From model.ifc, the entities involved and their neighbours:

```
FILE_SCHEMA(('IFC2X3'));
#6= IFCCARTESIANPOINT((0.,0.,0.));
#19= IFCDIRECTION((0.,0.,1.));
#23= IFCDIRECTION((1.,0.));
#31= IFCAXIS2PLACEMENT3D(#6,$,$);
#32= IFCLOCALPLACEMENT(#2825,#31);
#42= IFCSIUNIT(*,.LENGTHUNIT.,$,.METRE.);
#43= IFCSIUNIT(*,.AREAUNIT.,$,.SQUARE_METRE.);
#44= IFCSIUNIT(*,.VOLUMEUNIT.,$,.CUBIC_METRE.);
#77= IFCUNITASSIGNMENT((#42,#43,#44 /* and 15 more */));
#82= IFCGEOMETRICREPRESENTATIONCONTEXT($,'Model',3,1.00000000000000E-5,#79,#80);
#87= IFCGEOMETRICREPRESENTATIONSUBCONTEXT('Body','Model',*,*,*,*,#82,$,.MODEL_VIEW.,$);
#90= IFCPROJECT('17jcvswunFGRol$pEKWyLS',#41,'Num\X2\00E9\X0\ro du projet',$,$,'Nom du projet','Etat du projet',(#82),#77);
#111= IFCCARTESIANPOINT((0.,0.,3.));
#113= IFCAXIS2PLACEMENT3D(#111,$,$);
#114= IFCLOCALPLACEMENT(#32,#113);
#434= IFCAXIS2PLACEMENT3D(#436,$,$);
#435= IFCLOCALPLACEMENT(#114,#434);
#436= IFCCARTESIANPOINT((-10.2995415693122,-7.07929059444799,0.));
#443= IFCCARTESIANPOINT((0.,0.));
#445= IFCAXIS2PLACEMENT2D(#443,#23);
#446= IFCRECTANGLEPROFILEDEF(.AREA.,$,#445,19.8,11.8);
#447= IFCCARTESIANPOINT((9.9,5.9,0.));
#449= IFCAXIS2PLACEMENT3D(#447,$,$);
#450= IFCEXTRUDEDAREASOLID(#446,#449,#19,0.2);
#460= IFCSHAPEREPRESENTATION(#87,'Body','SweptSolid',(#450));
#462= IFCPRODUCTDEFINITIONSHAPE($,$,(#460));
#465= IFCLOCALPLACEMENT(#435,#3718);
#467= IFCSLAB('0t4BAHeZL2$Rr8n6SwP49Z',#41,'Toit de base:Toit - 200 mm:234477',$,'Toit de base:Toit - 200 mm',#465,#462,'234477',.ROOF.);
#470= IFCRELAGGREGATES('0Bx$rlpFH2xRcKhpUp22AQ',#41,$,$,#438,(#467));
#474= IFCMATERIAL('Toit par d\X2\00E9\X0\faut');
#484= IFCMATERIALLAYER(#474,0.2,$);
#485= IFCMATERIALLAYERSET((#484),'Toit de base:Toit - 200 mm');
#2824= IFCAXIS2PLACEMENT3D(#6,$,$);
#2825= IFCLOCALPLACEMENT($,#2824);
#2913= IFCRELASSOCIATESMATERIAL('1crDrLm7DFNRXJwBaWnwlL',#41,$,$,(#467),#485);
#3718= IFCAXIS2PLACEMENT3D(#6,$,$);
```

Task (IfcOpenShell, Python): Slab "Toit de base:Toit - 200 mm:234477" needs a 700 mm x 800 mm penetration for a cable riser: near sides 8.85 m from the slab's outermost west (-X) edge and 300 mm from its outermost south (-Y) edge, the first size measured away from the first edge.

```python
import numpy as np
import ifcopenshell
import ifcopenshell.api.feature
import ifcopenshell.api.geometry
import ifcopenshell.api.root
import ifcopenshell.geom
import ifcopenshell.util.placement
import ifcopenshell.util.representation
import ifcopenshell.util.shape
import ifcopenshell.util.unit

model = ifcopenshell.open("model.ifc")
unit_scale = ifcopenshell.util.unit.calculate_unit_scale(model)
settings = ifcopenshell.geom.settings()


def volume(element):
    """Net volume in cubic metres, openings subtracted."""
    shape = ifcopenshell.geom.create_shape(settings, element)
    return ifcopenshell.util.shape.get_volume(shape.geometry)


slab = model.by_id(467)
before = volume(slab)

# Extent in the slab's own axes, in metres. The edges named are its -X and -Y sides.
slab_shape = ifcopenshell.geom.create_shape(settings, slab)
vertices = ifcopenshell.util.shape.get_vertices(slab_shape.geometry)
x_min, y_min, bottom = vertices.min(axis=0)
top = vertices[:, 2].max()

opening = ifcopenshell.api.root.create_entity(model, ifc_class="IfcOpeningElement", name="Cable riser opening")
context = ifcopenshell.util.representation.get_context(model, "Model", "Body", "MODEL_VIEW")
width, depth = 0.7, 0.8
outline = [(0.0, 0.0), (width, 0.0), (width, depth), (0.0, depth), (0.0, 0.0)]
# Overshoot both faces by 50 mm so the cut is clean.
shape = ifcopenshell.api.geometry.add_slab_representation(
    model, context=context, depth=top - bottom + 0.1, polyline=outline
)
ifcopenshell.api.geometry.assign_representation(model, product=opening, representation=shape)

matrix = ifcopenshell.util.placement.get_local_placement(slab.ObjectPlacement)
matrix[:, 3] = matrix @ np.append(np.array([x_min + 8.85, y_min + 0.3, bottom - 0.05]) / unit_scale, 1.0)
ifcopenshell.api.geometry.edit_object_placement(model, product=opening, matrix=matrix, is_si=False)
ifcopenshell.api.feature.add_feature(model, feature=opening, element=slab)

after = volume(slab)

print(f"slab volume {before:.3f} -> {after:.3f} m3")

model.write("model-out.ifc")
```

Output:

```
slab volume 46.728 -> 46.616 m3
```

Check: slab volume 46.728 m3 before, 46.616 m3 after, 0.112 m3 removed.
